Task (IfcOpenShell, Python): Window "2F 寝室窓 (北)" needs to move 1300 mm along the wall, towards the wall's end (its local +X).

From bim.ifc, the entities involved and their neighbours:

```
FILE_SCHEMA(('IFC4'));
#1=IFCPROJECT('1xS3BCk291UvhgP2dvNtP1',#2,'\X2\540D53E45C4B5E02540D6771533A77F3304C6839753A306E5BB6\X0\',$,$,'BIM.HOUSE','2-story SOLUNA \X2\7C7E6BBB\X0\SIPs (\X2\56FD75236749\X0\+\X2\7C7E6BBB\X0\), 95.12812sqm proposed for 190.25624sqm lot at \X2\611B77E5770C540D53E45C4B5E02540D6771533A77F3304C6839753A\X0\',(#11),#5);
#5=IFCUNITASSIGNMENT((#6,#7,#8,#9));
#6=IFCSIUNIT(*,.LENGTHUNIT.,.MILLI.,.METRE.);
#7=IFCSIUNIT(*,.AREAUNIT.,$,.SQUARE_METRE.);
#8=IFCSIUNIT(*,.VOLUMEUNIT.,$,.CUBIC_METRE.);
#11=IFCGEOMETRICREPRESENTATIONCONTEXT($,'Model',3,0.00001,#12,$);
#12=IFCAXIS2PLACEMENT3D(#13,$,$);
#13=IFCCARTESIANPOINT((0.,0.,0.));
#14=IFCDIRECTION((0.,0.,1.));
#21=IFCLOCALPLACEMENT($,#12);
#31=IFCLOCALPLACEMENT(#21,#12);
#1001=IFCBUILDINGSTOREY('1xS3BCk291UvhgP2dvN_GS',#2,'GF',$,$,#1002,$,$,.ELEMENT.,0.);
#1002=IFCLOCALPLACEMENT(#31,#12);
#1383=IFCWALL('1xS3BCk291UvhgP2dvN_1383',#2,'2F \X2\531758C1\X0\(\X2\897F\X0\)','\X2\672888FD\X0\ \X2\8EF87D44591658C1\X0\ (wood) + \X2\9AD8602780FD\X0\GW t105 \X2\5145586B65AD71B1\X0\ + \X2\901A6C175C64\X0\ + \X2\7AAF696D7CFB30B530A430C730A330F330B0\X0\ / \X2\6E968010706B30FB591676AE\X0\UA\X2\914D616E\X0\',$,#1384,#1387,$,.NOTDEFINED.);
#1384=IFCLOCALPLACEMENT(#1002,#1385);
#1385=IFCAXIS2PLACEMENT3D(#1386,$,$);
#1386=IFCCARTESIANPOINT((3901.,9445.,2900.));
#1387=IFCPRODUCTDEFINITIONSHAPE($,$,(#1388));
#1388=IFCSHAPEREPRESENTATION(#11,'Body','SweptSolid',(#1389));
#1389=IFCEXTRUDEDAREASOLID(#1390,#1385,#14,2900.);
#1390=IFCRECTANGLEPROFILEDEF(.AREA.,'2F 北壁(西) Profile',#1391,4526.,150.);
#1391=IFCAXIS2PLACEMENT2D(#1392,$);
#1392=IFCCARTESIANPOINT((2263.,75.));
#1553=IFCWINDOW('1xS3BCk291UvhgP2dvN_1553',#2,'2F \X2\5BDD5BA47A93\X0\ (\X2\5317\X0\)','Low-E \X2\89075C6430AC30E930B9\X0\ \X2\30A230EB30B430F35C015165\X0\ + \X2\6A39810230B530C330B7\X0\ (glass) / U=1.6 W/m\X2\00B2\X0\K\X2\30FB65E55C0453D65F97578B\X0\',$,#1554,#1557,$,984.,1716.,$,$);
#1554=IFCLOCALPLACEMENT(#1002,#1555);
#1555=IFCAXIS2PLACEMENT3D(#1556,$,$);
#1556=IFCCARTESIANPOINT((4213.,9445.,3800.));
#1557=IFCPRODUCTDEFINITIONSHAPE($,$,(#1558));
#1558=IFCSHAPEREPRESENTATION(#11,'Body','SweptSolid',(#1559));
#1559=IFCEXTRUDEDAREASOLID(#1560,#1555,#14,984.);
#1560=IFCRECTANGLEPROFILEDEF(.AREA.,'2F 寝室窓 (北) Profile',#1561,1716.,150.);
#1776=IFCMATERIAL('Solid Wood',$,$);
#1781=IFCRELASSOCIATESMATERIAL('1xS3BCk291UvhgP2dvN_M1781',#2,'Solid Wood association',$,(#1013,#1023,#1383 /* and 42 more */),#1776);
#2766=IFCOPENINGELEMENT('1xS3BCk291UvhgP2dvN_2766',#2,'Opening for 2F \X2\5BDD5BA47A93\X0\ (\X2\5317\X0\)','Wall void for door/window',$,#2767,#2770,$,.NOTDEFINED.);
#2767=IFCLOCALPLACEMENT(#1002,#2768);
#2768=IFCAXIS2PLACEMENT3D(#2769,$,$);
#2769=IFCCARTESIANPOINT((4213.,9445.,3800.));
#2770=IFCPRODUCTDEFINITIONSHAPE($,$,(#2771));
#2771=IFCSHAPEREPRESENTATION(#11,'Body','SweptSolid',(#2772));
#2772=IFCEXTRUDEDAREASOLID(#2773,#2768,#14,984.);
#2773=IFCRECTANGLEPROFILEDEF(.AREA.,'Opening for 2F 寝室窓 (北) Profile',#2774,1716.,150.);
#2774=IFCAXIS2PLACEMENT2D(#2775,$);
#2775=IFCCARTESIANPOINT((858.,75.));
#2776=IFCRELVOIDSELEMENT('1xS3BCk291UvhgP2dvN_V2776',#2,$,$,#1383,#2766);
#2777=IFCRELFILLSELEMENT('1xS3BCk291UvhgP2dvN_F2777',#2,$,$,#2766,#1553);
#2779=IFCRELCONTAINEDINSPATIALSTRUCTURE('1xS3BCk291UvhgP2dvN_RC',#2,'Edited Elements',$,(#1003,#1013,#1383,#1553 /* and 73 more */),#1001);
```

```python
import ifcopenshell
import ifcopenshell.api.geometry
import ifcopenshell.util.placement
import ifcopenshell.util.unit

model = ifcopenshell.open("bim.ifc")
unit_scale = ifcopenshell.util.unit.calculate_unit_scale(model)

window = model.by_guid("1xS3BCk291UvhgP2dvN_1553")
opening = window.FillsVoids[0].RelatingOpeningElement
wall = opening.VoidsElements[0].RelatingBuildingElement

wall_matrix = ifcopenshell.util.placement.get_local_placement(wall.ObjectPlacement)
shift = wall_matrix[:3, 0] * 1.3 / unit_scale
before = ifcopenshell.util.placement.get_local_placement(window.ObjectPlacement)[:3, 3].copy()

# The window is not placed relative to its opening, so move both.
for product in (opening, window):
    matrix = ifcopenshell.util.placement.get_local_placement(product.ObjectPlacement)
    matrix[:3, 3] += shift
    ifcopenshell.api.geometry.edit_object_placement(model, product=product, matrix=matrix, is_si=False)

after = ifcopenshell.util.placement.get_local_placement(window.ObjectPlacement)[:3, 3]
print("window moved by", (after - before).round(3) + 0.0)

model.write("bim-out.ifc")
```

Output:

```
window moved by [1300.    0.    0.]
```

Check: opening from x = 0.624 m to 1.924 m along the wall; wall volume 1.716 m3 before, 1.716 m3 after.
